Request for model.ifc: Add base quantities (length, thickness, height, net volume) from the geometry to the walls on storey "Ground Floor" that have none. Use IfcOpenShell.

First a look at what the model holds.

```python
import ifcopenshell
import ifcopenshell.util.element
import ifcopenshell.util.unit

model = ifcopenshell.open("model.ifc")
print(model.schema)
for unit_type in ("LENGTHUNIT", "AREAUNIT", "VOLUMEUNIT"):
    print(unit_type, ifcopenshell.util.unit.calculate_unit_scale(model, unit_type))
storey = next(s for s in model.by_type("IfcBuildingStorey") if s.Name == "Ground Floor")
walls = [e for e in ifcopenshell.util.element.get_decomposition(storey) if e.is_a("IfcWall")]
for e in sorted(walls, key=lambda e: e.id()):
    print(e.id(), e.is_a(), e.Name, list(ifcopenshell.util.element.get_psets(e, qtos_only=True)), sep=" | ")
```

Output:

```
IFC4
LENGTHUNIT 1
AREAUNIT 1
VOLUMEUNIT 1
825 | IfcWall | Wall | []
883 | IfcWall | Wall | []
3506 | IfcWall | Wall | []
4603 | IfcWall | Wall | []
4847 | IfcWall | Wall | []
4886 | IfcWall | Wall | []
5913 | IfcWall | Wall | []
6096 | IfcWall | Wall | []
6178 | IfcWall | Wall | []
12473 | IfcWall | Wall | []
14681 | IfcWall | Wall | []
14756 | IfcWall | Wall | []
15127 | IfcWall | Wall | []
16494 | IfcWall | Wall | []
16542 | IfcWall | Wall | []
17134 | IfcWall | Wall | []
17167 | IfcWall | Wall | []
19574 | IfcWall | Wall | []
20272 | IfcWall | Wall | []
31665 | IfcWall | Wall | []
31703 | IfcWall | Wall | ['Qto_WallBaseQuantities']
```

```python
import ifcopenshell
import ifcopenshell.api.pset
import ifcopenshell.geom
import ifcopenshell.util.element
import ifcopenshell.util.shape
import ifcopenshell.util.unit

model = ifcopenshell.open("model.ifc")
unit_scale = ifcopenshell.util.unit.calculate_unit_scale(model)
volume_scale = ifcopenshell.util.unit.calculate_unit_scale(model, "VOLUMEUNIT")
settings = ifcopenshell.geom.settings()

storey = next(s for s in model.by_type("IfcBuildingStorey") if s.Name == "Ground Floor")
walls = [e for e in ifcopenshell.util.element.get_decomposition(storey) if e.is_a("IfcWall")]

for e in sorted(walls, key=lambda e: e.id()):
    if ifcopenshell.util.element.get_psets(e, qtos_only=True, should_inherit=False):
        continue
    # Geometry comes back in metres, in the element's own axes.
    shape = ifcopenshell.geom.create_shape(settings, e)
    values = {
        "Length": ifcopenshell.util.shape.get_x(shape.geometry) / unit_scale,
        "Width": ifcopenshell.util.shape.get_y(shape.geometry) / unit_scale,
        "Height": ifcopenshell.util.shape.get_z(shape.geometry) / unit_scale,
        "NetVolume": ifcopenshell.util.shape.get_volume(shape.geometry) / volume_scale,
    }
    qto = ifcopenshell.api.pset.add_qto(model, product=e, name="Qto_WallBaseQuantities")
    ifcopenshell.api.pset.edit_qto(model, qto=qto, properties=values)
    print(e.id(), {k: round(v, 3) for k, v in values.items()})

model.write("model_v2.ifc")
```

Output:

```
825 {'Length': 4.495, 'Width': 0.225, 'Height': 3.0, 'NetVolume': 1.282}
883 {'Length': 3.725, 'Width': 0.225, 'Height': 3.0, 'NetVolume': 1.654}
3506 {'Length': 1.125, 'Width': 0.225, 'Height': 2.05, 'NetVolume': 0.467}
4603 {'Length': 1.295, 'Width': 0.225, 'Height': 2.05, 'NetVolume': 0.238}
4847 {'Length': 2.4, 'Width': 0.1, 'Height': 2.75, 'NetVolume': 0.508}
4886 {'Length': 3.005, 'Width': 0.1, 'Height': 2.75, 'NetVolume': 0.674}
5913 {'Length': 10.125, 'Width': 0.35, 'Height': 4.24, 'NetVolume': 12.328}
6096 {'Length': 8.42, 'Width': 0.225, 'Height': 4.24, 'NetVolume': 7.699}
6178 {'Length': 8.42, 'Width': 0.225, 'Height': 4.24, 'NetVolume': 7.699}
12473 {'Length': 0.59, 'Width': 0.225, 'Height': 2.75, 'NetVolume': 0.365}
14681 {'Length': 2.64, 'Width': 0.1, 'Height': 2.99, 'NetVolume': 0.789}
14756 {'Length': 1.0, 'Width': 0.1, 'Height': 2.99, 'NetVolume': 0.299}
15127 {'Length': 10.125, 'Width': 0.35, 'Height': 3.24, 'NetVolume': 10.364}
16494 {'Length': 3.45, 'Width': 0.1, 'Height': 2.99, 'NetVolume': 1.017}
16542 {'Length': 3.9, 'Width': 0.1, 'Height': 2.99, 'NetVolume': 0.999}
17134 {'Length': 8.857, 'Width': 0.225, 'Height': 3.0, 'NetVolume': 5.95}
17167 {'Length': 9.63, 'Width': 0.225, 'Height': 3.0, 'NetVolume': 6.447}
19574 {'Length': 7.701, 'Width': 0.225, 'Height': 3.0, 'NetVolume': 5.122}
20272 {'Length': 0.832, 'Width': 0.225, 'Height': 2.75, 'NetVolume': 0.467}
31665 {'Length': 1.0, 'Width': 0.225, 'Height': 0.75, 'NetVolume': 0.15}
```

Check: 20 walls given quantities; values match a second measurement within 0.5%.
